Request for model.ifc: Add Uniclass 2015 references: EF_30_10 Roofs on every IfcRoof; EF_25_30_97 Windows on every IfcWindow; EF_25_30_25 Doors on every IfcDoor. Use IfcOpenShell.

First a look at what the model holds.

```python
import ifcopenshell

model = ifcopenshell.open("model.ifc")
print(model.schema)
print("classifications:", [c.Name for c in model.by_type("IfcClassification")])
for ifc_class in ("IfcDoor", "IfcRoof", "IfcStair", "IfcWall", "IfcWindow"):
    print(ifc_class, len(model.by_type(ifc_class)))
```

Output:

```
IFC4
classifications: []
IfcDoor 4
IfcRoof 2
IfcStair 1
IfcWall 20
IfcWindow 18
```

```python
import ifcopenshell
import ifcopenshell.api.classification

model = ifcopenshell.open("model.ifc")

system = ifcopenshell.api.classification.add_classification(model, classification="Uniclass 2015")

codes = {
    "IfcRoof": ("EF_30_10", "Roofs"),
    "IfcWindow": ("EF_25_30_97", "Windows"),
    "IfcDoor": ("EF_25_30_25", "Doors"),
}
for ifc_class, (code, name) in codes.items():
    products = model.by_type(ifc_class)
    ifcopenshell.api.classification.add_reference(
        model, products=products, classification=system, identification=code, name=name
    )
    print(code, len(products))

model.write("model_rev.ifc")
```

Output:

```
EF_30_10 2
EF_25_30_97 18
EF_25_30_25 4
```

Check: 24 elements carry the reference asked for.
